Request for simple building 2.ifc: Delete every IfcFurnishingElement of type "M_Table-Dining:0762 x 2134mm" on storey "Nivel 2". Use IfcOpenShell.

First a look at what the model holds.

```python
import ifcopenshell
import ifcopenshell.util.element

model = ifcopenshell.open("simple building 2.ifc")
print(model.schema)
storey = next(s for s in model.by_type("IfcBuildingStorey") if s.Name == "Nivel 2")
furniture = [e for e in ifcopenshell.util.element.get_decomposition(storey) if e.is_a("IfcFurnishingElement")]
seen = {}
for e in furniture:
    element_type = ifcopenshell.util.element.get_type(e)
    name = element_type.Name if element_type not in (None, e) else None
    seen[name] = seen.get(name, 0) + 1
for name, count in sorted(seen.items(), key=str):
    print(count, "x", name)
```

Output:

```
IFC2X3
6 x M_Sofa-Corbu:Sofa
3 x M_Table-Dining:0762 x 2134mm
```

```python
import ifcopenshell
import ifcopenshell.api.root
import ifcopenshell.util.element

model = ifcopenshell.open("simple building 2.ifc")

storey = next(s for s in model.by_type("IfcBuildingStorey") if s.Name == "Nivel 2")
furniture = [e for e in ifcopenshell.util.element.get_decomposition(storey) if e.is_a("IfcFurnishingElement")]
targets = [e for e in furniture if (t := ifcopenshell.util.element.get_type(e)) not in (None, e) and t.Name == "M_Table-Dining:0762 x 2134mm"]

for e in targets:
    ifcopenshell.api.root.remove_product(model, product=e)
print(len(targets), "removed")

model.write("simple building 2_edited.ifc")
```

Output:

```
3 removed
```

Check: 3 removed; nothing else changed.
